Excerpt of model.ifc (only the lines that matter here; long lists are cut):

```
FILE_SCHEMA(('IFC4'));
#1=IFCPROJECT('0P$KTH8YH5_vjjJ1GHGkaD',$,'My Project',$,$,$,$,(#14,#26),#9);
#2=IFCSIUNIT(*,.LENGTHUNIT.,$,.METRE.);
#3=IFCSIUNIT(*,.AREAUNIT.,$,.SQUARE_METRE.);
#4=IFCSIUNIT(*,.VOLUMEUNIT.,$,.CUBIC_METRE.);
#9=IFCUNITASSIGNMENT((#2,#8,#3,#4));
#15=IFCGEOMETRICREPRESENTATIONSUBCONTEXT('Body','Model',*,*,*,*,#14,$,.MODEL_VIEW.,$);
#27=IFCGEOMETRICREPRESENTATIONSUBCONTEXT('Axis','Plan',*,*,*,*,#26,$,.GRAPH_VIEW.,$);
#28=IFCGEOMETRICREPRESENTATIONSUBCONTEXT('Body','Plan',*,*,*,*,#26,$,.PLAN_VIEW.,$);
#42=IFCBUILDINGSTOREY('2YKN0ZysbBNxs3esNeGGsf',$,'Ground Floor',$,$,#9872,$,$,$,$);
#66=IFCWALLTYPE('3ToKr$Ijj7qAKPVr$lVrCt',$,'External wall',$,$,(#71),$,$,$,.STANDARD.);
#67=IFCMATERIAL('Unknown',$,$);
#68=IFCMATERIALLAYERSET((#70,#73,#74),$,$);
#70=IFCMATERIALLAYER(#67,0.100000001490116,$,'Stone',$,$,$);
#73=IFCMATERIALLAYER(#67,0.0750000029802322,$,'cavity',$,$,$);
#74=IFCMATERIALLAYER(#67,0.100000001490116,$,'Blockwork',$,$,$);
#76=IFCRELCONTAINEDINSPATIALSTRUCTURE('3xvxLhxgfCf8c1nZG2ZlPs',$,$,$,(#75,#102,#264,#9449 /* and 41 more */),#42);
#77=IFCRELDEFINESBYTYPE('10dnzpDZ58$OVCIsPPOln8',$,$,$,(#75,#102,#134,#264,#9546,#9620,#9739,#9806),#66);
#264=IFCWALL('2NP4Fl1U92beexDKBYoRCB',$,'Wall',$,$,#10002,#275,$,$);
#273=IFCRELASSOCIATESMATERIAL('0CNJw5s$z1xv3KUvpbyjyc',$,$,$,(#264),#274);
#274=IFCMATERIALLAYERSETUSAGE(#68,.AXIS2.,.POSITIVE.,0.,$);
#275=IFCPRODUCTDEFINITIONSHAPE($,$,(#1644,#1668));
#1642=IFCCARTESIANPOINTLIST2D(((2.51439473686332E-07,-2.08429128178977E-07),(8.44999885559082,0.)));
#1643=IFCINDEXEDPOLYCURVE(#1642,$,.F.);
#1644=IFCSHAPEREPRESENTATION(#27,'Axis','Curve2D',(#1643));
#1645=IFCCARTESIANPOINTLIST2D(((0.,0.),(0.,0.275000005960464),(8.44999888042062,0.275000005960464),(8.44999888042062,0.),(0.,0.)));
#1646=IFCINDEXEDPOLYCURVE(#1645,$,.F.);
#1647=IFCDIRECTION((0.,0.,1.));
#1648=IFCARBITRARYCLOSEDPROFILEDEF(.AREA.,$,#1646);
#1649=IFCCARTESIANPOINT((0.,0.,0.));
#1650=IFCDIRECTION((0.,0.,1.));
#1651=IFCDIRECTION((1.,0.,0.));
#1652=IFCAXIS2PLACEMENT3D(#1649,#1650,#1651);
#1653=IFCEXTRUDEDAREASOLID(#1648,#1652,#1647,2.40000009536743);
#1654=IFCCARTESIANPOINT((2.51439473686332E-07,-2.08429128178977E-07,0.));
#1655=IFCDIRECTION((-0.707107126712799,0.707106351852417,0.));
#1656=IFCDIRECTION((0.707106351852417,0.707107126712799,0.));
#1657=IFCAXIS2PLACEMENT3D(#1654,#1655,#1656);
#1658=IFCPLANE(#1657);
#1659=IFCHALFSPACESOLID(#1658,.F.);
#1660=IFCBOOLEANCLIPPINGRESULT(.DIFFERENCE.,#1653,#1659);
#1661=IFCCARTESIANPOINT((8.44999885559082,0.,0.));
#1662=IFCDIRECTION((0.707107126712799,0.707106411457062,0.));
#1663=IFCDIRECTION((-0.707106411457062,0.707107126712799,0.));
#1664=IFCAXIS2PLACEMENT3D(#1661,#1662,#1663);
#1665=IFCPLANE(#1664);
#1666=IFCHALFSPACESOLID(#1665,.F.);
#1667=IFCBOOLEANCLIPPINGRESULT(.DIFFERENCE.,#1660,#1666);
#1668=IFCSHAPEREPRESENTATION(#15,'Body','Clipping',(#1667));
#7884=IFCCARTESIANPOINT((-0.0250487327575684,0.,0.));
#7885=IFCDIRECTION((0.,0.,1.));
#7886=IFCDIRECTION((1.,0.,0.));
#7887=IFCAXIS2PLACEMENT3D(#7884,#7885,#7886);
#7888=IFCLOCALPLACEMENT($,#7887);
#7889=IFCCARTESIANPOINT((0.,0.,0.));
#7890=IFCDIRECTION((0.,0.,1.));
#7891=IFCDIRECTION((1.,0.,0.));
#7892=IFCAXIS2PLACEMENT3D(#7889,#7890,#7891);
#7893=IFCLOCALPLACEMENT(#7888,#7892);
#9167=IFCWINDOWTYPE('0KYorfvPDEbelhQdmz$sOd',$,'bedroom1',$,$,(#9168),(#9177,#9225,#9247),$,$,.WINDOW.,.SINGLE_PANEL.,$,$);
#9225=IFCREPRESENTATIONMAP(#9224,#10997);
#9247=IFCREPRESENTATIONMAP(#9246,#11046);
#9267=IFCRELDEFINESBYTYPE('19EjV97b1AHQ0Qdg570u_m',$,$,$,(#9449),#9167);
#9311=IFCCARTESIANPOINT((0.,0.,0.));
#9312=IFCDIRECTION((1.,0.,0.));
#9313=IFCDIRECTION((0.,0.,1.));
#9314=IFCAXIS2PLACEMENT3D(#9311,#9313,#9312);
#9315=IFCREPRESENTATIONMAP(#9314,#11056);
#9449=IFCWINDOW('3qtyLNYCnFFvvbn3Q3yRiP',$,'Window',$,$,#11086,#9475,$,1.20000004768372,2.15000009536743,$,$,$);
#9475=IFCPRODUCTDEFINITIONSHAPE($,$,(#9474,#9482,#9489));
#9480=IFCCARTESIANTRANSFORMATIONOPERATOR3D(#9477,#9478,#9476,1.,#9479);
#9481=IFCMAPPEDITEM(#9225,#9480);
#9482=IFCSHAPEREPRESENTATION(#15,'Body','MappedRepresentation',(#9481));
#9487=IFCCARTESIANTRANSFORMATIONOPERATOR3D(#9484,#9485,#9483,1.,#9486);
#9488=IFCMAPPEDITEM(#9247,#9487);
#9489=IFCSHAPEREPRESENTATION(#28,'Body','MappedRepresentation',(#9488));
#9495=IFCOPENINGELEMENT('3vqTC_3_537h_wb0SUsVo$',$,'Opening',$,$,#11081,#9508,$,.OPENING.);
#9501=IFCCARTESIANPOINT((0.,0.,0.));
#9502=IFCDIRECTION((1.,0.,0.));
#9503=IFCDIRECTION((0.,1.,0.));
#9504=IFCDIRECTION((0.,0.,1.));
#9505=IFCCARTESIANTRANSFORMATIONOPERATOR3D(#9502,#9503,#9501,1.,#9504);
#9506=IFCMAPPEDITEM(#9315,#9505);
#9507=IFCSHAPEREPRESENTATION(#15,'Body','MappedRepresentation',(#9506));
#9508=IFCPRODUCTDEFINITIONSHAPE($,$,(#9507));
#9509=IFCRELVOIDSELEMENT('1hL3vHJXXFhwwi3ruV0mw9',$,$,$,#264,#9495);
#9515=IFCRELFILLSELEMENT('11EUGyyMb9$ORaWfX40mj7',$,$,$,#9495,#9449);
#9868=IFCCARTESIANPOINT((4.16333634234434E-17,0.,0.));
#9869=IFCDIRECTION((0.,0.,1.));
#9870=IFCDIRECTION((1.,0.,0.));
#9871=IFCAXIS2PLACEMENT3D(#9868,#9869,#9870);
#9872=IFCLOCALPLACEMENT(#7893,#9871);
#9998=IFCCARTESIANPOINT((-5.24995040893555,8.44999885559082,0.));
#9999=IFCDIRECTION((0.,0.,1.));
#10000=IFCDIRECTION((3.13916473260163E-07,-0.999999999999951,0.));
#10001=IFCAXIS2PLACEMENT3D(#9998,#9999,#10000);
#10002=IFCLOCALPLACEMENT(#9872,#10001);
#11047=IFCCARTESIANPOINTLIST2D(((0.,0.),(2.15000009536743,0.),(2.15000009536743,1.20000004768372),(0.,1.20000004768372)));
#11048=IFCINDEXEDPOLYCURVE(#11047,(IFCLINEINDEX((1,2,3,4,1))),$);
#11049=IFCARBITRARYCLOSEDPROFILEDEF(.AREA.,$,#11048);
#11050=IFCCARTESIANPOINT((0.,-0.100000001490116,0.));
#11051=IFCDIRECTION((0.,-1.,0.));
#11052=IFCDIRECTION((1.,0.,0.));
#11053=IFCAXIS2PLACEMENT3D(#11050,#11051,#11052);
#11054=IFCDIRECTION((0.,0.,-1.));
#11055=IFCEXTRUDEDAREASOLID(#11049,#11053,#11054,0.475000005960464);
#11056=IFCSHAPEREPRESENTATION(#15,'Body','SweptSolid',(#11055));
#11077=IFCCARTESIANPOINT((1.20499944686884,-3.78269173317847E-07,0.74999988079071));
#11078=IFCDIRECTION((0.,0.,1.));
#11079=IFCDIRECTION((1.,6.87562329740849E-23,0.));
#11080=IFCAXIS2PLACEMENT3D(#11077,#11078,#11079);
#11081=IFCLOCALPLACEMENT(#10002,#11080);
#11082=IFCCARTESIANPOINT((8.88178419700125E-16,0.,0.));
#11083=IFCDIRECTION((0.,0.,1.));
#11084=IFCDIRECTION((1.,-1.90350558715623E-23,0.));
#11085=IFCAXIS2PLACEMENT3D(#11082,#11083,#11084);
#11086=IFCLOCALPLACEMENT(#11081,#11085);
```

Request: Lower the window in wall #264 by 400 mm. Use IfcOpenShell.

```python
import numpy as np
import ifcopenshell
import ifcopenshell.api.geometry
import ifcopenshell.util.placement
import ifcopenshell.util.unit

model = ifcopenshell.open("model.ifc")
unit_scale = ifcopenshell.util.unit.calculate_unit_scale(model)

window = model.by_guid("3qtyLNYCnFFvvbn3Q3yRiP")
opening = window.FillsVoids[0].RelatingOpeningElement
dz = -0.4

shift = np.array([0.0, 0.0, dz])
# The window is placed relative to its opening, so it follows when the opening moves.
matrix = ifcopenshell.util.placement.get_local_placement(opening.ObjectPlacement)
matrix[:3, 3] += shift
ifcopenshell.api.geometry.edit_object_placement(
    model, product=opening, matrix=matrix, is_si=False, should_transform_children=True
)

print(f"moved by {dz * unit_scale:+.3f} m")

model.write("model_edited.ifc")
```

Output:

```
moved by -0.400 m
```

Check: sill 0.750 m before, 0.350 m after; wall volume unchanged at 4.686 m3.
